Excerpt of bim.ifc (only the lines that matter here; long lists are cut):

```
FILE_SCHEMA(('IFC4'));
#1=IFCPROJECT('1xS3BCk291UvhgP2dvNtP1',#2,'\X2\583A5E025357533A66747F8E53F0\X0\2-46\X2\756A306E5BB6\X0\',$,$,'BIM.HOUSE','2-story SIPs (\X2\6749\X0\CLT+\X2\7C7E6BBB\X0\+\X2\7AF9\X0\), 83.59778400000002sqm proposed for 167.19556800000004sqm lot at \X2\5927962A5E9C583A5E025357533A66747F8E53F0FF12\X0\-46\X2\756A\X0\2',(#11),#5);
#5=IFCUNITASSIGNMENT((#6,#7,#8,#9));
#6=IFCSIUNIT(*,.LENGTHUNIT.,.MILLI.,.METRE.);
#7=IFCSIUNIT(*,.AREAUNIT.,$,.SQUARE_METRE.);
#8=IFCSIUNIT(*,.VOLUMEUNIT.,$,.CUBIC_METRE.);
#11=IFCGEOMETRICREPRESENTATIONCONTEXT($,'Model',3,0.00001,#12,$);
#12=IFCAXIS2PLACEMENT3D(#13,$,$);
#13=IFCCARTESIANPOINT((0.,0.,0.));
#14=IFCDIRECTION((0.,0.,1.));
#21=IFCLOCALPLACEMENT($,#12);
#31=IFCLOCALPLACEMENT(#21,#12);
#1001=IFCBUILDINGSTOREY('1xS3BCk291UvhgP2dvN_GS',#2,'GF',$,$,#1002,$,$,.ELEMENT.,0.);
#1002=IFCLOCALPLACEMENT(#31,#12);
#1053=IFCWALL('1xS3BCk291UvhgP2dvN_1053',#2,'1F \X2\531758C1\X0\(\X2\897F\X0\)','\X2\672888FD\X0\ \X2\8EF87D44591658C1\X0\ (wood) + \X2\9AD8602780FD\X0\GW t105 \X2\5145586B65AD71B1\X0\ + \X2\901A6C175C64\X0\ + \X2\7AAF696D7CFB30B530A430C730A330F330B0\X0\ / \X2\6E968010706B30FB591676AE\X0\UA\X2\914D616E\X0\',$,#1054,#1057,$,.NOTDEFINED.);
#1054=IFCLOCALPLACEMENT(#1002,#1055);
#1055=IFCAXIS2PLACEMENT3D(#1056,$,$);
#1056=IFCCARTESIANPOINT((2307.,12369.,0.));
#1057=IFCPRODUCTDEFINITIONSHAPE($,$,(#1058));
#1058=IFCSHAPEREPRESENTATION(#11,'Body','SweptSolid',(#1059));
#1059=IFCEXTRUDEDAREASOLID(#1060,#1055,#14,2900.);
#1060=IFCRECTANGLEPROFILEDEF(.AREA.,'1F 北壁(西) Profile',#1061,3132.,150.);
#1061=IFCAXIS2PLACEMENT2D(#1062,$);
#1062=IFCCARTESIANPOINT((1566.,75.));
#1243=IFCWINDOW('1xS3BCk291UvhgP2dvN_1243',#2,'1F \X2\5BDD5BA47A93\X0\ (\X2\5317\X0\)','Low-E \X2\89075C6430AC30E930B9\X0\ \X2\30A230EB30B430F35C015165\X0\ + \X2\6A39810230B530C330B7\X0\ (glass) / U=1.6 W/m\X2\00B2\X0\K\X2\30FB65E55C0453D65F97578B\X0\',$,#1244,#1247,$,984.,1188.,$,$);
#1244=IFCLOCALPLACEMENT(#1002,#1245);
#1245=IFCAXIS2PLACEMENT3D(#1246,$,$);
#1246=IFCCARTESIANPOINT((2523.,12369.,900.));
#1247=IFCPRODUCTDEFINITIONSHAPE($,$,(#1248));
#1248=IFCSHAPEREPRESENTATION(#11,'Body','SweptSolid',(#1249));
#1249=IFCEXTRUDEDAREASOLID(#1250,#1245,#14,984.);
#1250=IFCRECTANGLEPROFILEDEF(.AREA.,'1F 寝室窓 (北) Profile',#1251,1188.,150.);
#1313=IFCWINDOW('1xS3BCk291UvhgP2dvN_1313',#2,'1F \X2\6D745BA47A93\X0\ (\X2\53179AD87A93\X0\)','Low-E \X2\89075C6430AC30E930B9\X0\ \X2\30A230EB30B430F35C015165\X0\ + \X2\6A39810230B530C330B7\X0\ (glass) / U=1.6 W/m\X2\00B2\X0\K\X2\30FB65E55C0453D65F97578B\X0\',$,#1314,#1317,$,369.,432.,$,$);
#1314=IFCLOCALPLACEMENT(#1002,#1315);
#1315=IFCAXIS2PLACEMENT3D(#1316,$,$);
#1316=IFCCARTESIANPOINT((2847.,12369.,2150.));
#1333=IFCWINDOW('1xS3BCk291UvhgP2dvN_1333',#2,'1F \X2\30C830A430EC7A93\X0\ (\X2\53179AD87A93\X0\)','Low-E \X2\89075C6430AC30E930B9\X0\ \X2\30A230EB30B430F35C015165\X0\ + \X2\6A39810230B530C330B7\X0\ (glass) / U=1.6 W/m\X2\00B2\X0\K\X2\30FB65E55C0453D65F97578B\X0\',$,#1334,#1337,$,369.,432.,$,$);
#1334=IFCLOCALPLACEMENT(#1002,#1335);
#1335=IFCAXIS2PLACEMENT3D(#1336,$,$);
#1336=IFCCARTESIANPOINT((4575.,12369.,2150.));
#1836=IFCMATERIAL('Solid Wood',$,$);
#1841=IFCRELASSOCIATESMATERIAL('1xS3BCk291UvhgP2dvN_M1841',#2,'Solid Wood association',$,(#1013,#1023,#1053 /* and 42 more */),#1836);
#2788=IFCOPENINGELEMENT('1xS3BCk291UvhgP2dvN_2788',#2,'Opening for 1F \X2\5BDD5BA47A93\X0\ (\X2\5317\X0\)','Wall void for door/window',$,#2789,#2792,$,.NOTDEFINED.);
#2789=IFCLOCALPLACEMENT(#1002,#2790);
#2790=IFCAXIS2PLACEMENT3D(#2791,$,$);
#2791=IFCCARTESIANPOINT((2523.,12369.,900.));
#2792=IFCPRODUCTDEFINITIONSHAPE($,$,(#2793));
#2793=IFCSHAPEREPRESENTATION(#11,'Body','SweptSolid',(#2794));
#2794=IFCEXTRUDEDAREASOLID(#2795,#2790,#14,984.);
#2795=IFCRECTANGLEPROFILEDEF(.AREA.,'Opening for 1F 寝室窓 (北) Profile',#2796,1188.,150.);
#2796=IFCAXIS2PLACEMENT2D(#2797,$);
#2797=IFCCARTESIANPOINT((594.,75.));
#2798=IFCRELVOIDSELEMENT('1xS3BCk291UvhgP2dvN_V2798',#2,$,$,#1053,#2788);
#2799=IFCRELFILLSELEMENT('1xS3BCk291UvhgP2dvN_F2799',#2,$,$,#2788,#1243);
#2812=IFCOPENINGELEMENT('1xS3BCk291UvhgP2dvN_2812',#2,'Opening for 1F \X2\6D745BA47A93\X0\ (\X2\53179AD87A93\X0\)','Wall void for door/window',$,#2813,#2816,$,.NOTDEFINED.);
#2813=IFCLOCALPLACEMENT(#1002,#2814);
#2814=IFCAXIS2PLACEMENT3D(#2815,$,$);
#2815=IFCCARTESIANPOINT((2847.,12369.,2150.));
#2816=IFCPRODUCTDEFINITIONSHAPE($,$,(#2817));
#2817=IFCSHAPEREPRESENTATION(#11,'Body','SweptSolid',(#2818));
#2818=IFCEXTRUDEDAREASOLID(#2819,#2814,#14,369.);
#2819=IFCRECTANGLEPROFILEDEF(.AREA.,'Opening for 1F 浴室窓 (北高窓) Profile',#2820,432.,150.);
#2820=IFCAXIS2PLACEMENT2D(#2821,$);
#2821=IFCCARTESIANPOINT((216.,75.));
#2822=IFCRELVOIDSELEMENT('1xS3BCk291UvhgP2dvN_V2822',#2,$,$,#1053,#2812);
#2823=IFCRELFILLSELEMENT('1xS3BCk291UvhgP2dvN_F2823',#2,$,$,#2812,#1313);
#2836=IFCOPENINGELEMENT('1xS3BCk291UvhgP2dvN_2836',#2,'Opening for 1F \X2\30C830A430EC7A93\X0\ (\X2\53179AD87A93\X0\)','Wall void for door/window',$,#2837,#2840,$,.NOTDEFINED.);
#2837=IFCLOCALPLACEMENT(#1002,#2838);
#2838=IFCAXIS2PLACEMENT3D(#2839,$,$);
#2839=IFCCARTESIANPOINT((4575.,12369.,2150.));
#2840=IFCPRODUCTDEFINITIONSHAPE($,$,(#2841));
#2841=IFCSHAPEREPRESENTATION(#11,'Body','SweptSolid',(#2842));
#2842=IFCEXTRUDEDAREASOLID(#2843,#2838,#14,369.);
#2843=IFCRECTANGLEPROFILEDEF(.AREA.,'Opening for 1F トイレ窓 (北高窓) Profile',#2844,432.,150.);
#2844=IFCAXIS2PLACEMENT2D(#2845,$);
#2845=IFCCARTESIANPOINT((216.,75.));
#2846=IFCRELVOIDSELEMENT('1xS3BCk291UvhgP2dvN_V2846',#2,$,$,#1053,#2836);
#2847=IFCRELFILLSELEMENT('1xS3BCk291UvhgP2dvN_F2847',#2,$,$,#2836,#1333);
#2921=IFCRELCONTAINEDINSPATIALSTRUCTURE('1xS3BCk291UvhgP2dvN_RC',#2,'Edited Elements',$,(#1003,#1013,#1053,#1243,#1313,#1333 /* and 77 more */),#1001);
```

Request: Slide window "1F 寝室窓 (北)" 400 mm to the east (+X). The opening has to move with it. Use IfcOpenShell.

```python
import ifcopenshell
import ifcopenshell.api.geometry
import ifcopenshell.util.placement
import ifcopenshell.util.unit

model = ifcopenshell.open("bim.ifc")
unit_scale = ifcopenshell.util.unit.calculate_unit_scale(model)

window = model.by_id(1243)
opening = window.FillsVoids[0].RelatingOpeningElement
wall = opening.VoidsElements[0].RelatingBuildingElement

wall_matrix = ifcopenshell.util.placement.get_local_placement(wall.ObjectPlacement)
shift = wall_matrix[:3, 0] * 0.4 / unit_scale
before = ifcopenshell.util.placement.get_local_placement(window.ObjectPlacement)[:3, 3].copy()

# The window is not placed relative to its opening, so move both.
for product in (opening, window):
    matrix = ifcopenshell.util.placement.get_local_placement(product.ObjectPlacement)
    matrix[:3, 3] += shift
    ifcopenshell.api.geometry.edit_object_placement(model, product=product, matrix=matrix, is_si=False)

after = ifcopenshell.util.placement.get_local_placement(window.ObjectPlacement)[:3, 3]
print("window moved by", (after - before).round(3) + 0.0)

model.write("bim_edited.ifc")
```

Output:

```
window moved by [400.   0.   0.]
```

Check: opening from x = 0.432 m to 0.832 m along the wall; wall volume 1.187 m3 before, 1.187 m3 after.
